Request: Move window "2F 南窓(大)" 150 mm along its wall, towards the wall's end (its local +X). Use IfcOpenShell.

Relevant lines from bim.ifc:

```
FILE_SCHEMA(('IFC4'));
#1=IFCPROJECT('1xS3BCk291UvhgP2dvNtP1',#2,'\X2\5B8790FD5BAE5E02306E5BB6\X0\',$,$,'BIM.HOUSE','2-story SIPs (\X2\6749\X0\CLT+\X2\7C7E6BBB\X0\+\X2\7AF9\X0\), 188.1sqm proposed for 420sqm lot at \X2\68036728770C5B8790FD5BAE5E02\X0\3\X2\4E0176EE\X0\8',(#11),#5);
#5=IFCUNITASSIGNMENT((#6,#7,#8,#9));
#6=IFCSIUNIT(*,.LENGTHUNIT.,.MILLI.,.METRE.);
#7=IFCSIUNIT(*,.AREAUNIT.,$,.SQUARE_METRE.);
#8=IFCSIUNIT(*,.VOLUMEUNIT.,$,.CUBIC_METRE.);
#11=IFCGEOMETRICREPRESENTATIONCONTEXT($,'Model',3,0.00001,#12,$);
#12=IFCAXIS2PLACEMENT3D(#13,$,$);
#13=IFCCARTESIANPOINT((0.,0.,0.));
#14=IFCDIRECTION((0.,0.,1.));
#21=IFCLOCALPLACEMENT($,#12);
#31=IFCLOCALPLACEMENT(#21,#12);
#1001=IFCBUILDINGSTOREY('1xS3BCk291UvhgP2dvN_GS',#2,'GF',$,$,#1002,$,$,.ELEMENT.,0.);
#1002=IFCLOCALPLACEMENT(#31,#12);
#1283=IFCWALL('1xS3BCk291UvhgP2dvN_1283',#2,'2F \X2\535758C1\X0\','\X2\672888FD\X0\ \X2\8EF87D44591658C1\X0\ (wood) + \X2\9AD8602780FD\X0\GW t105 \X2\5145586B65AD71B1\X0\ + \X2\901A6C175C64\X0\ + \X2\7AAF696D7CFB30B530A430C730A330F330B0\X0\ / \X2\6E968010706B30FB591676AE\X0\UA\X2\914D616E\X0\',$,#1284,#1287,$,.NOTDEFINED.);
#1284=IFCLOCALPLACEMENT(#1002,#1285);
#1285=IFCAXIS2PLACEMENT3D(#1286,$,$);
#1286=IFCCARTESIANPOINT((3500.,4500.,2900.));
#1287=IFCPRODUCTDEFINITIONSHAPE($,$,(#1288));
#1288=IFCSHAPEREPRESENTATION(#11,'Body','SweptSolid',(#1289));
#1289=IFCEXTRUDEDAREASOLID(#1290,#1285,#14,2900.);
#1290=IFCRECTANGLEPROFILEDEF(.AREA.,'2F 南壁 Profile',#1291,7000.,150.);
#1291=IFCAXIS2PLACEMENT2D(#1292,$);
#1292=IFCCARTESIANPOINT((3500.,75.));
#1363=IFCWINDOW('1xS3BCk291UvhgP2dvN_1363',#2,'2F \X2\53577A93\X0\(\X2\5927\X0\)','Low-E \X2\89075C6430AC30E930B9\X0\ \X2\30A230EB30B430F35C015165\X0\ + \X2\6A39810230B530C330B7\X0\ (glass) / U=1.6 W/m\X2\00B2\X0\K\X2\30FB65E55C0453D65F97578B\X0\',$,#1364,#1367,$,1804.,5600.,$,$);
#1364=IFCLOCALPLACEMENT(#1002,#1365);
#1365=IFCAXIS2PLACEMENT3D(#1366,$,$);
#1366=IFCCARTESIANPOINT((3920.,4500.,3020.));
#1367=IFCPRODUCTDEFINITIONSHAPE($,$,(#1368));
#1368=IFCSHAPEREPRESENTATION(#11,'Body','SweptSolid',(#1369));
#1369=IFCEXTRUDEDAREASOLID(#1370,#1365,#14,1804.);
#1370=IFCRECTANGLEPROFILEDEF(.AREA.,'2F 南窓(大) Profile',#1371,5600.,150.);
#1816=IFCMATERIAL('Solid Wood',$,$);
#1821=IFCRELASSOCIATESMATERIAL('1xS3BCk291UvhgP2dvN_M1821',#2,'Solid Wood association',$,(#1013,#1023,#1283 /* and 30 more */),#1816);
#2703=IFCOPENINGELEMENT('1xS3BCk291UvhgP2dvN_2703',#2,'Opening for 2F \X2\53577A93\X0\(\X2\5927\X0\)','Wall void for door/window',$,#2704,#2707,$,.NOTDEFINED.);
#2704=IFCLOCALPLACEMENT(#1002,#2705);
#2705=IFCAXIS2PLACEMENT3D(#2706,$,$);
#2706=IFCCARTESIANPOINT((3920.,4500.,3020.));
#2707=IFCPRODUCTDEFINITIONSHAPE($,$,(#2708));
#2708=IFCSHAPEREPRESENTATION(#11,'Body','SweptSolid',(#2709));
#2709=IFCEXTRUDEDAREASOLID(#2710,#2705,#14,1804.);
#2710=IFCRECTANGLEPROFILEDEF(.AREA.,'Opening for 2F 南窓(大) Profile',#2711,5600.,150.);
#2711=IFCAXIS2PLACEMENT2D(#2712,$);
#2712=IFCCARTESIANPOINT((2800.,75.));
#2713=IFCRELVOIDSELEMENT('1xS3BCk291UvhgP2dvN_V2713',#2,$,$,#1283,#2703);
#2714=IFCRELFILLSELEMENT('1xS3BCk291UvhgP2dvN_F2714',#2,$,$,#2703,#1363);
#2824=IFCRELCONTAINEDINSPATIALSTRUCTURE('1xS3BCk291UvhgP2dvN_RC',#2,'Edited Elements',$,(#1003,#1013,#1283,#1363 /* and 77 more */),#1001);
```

```python
import ifcopenshell
import ifcopenshell.api.geometry
import ifcopenshell.util.placement
import ifcopenshell.util.unit

model = ifcopenshell.open("bim.ifc")
unit_scale = ifcopenshell.util.unit.calculate_unit_scale(model)

window = model.by_guid("1xS3BCk291UvhgP2dvN_1363")
opening = window.FillsVoids[0].RelatingOpeningElement
wall = opening.VoidsElements[0].RelatingBuildingElement

wall_matrix = ifcopenshell.util.placement.get_local_placement(wall.ObjectPlacement)
shift = wall_matrix[:3, 0] * 0.15 / unit_scale
before = ifcopenshell.util.placement.get_local_placement(window.ObjectPlacement)[:3, 3].copy()

# The window is not placed relative to its opening, so move both.
for product in (opening, window):
    matrix = ifcopenshell.util.placement.get_local_placement(product.ObjectPlacement)
    matrix[:3, 3] += shift
    ifcopenshell.api.geometry.edit_object_placement(model, product=product, matrix=matrix, is_si=False)

after = ifcopenshell.util.placement.get_local_placement(window.ObjectPlacement)[:3, 3]
print("window moved by", (after - before).round(3) + 0.0)

model.write("bim_v2.ifc")
```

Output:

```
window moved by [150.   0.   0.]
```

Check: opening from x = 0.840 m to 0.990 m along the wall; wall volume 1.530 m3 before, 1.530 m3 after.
